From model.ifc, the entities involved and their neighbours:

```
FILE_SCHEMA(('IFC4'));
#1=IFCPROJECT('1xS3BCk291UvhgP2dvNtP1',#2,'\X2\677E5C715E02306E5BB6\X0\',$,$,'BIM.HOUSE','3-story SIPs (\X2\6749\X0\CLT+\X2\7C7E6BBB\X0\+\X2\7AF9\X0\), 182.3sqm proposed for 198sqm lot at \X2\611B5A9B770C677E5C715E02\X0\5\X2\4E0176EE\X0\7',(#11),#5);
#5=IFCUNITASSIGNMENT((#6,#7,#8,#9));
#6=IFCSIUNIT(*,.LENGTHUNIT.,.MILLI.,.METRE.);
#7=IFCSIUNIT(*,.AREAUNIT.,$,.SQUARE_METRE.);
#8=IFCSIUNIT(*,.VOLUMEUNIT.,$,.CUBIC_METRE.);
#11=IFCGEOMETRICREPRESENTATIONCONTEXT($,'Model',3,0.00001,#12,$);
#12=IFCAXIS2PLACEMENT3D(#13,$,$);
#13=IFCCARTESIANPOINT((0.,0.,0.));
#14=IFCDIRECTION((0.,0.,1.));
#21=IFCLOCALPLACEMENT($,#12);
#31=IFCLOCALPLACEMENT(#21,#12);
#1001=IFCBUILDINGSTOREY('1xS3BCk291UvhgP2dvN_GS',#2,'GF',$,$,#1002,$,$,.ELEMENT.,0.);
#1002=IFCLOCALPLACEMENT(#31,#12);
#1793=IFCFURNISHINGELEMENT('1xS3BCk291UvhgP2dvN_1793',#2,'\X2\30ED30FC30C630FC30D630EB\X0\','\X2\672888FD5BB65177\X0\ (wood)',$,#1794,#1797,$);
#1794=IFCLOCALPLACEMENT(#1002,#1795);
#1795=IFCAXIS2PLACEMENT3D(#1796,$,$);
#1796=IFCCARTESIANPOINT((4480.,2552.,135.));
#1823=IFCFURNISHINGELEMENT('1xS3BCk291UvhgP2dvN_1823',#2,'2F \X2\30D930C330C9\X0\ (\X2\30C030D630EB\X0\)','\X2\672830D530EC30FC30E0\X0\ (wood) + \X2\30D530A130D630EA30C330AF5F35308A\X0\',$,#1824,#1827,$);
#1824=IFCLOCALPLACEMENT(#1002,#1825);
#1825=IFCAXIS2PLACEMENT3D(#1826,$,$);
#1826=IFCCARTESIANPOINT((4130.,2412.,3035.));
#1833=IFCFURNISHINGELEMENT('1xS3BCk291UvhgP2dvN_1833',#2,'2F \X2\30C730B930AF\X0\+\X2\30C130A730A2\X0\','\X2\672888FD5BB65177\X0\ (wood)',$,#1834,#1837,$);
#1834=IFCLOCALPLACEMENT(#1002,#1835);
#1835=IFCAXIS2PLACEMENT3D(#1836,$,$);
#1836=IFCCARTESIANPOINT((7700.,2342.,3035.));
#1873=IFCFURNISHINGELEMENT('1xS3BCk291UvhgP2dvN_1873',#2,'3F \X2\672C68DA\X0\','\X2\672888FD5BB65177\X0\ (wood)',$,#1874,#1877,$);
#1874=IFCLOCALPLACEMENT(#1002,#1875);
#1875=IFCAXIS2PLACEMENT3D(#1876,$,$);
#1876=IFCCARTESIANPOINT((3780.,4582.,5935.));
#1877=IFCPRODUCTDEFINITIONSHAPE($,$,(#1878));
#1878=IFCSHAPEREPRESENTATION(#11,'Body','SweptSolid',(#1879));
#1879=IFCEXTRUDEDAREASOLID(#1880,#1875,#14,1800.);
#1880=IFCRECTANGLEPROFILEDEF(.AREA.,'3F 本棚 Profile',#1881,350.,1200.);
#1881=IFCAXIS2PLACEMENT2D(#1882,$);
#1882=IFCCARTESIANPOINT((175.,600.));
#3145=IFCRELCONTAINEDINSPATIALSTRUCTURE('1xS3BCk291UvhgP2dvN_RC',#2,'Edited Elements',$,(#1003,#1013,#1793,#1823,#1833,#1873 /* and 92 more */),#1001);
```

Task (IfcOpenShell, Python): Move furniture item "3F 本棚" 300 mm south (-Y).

```python
import ifcopenshell
import ifcopenshell.api.geometry
import ifcopenshell.util.placement
import ifcopenshell.util.unit

model = ifcopenshell.open("model.ifc")
unit_scale = ifcopenshell.util.unit.calculate_unit_scale(model)

item = model.by_guid("1xS3BCk291UvhgP2dvN_1873")
matrix = ifcopenshell.util.placement.get_local_placement(item.ObjectPlacement)
matrix[1, 3] -= 0.3 / unit_scale
ifcopenshell.api.geometry.edit_object_placement(model, product=item, matrix=matrix, is_si=False)

print(ifcopenshell.util.placement.get_local_placement(item.ObjectPlacement).round(3) + 0.0)

model.write("model-out.ifc")
```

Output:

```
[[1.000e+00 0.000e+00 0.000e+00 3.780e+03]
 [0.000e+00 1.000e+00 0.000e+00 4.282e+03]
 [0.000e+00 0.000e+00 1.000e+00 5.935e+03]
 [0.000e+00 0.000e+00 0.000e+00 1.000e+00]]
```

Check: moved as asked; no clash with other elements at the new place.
